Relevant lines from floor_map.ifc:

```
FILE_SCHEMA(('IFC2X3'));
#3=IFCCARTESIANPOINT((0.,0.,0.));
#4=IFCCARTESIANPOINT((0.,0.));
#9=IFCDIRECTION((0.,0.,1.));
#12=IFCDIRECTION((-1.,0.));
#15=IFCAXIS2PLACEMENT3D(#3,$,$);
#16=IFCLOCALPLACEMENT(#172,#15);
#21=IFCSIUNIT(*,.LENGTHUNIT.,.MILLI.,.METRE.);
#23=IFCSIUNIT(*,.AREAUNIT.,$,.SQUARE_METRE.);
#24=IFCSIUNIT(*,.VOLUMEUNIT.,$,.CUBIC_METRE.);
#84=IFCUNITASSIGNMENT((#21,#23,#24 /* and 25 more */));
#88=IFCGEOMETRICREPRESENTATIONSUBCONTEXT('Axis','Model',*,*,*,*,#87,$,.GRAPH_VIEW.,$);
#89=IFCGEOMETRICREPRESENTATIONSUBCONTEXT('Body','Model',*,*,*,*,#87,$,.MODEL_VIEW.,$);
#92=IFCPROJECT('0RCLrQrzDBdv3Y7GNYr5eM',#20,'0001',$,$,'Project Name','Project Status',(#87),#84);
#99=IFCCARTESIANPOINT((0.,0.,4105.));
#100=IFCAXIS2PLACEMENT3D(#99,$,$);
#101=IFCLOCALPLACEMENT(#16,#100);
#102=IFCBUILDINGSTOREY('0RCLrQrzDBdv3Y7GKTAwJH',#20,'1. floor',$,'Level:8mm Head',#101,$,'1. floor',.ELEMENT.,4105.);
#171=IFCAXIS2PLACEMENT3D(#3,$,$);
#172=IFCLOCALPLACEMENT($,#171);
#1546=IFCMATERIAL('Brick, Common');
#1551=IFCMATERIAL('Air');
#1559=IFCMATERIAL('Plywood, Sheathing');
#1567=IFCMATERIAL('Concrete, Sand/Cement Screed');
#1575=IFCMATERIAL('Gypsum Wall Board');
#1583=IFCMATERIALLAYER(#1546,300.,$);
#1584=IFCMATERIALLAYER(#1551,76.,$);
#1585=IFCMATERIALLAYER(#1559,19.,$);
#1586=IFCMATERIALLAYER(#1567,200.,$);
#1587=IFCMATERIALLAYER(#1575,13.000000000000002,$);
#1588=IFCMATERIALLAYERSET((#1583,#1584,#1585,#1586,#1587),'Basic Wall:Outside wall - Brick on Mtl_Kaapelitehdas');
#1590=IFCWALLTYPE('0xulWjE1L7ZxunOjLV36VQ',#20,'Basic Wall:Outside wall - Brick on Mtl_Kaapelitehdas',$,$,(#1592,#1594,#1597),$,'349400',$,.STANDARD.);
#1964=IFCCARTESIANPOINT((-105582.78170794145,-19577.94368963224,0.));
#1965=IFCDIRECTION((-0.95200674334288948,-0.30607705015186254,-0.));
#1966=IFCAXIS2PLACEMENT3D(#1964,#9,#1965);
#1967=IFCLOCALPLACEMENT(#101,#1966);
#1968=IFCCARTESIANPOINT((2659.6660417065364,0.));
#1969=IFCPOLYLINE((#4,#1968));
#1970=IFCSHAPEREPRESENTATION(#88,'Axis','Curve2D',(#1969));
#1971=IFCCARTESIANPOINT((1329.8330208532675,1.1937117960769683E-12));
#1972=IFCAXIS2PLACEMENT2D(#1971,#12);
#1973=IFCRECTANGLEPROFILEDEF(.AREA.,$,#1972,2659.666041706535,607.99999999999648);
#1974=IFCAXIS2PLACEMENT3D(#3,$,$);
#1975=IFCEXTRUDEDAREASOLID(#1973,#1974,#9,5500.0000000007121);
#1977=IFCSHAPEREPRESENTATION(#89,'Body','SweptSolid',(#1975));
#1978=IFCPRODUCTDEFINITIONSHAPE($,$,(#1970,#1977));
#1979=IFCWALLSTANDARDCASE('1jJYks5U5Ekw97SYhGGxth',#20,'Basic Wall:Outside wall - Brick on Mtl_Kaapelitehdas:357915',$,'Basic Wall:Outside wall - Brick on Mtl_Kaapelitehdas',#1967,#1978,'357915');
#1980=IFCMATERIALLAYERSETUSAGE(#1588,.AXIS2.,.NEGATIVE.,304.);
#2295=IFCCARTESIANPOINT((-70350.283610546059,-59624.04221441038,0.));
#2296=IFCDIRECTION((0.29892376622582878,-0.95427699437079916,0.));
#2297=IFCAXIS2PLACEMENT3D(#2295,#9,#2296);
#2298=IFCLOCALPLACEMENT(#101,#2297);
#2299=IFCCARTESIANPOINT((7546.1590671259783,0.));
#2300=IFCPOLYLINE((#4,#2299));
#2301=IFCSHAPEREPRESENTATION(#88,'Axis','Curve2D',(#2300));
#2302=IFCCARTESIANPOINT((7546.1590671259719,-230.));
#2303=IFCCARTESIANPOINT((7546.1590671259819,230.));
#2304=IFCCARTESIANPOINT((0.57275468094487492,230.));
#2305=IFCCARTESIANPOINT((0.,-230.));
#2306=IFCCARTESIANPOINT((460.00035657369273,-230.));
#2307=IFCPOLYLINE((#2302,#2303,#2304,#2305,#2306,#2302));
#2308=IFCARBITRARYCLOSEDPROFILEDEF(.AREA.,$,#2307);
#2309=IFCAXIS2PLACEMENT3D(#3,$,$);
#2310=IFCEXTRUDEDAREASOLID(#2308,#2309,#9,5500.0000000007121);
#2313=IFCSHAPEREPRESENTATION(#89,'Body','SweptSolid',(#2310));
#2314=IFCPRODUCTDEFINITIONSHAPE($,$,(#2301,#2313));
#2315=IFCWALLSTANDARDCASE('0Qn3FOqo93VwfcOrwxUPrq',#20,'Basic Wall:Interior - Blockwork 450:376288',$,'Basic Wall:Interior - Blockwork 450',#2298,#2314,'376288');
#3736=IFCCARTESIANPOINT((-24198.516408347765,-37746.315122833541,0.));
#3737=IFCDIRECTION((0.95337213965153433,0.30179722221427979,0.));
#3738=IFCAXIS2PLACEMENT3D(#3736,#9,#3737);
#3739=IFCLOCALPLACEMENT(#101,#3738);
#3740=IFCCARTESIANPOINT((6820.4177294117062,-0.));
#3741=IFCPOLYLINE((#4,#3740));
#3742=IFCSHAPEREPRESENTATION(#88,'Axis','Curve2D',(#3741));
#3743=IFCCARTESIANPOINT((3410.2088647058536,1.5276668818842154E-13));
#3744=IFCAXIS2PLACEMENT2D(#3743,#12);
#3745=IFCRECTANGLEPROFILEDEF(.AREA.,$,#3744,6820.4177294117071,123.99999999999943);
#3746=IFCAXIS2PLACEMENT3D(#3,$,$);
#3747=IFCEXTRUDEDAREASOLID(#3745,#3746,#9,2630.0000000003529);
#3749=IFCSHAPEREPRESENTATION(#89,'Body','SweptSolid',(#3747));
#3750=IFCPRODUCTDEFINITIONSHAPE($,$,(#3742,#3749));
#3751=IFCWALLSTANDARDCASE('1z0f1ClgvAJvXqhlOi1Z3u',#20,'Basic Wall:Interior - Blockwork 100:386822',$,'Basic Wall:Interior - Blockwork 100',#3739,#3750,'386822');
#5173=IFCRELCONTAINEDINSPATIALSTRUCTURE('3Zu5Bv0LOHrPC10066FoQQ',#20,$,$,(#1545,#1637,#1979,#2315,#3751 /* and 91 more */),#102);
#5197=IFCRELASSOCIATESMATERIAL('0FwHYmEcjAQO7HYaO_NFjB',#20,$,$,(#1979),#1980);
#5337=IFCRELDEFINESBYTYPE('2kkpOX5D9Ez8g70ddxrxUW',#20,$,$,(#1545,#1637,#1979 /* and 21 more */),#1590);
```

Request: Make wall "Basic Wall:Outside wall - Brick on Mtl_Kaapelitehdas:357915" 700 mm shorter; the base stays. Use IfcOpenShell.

```python
import ifcopenshell
import ifcopenshell.geom
import ifcopenshell.util.representation
import ifcopenshell.util.shape
import ifcopenshell.util.unit

model = ifcopenshell.open("floor_map.ifc")
unit_scale = ifcopenshell.util.unit.calculate_unit_scale(model)
settings = ifcopenshell.geom.settings()


def volume(element):
    """Net volume in cubic metres, openings subtracted."""
    shape = ifcopenshell.geom.create_shape(settings, element)
    return ifcopenshell.util.shape.get_volume(shape.geometry)


wall = model.by_id(1979)
before = volume(wall)

body = ifcopenshell.util.representation.get_representation(wall, "Model", "Body")
solid = body.Items[0]
old_height = solid.Depth
solid.Depth -= 0.7 / unit_scale
after = volume(wall)

print(f"height {old_height:g} -> {solid.Depth:g}, volume {before:.3f} -> {after:.3f} m3")

model.write("floor_map_updated.ifc")
```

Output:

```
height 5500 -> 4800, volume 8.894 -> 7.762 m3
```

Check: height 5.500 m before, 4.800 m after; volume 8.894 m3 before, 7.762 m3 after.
